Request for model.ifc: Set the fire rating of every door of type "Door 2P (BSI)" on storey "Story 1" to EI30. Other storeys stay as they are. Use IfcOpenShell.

First a look at what the model holds.

```python
import ifcopenshell
import ifcopenshell.util.element

model = ifcopenshell.open("model.ifc")
print(model.schema)
storey = next(s for s in model.by_type("IfcBuildingStorey") if s.Name == "Story 1")
doors = [e for e in ifcopenshell.util.element.get_decomposition(storey) if e.is_a("IfcDoor")]
seen = {}
for e in doors:
    element_type = ifcopenshell.util.element.get_type(e)
    key = (element_type.Name if element_type != e and element_type else None, ifcopenshell.util.element.get_pset(e, "Pset_DoorCommon", "FireRating"))
    seen[key] = seen.get(key, 0) + 1
for (name, value), count in sorted(seen.items(), key=str):
    print(count, "x", name, "|", value)
```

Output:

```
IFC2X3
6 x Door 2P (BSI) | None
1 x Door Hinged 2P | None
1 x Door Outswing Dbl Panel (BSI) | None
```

```python
import ifcopenshell
import ifcopenshell.api.pset
import ifcopenshell.util.element

model = ifcopenshell.open("model.ifc")

storey = next(s for s in model.by_type("IfcBuildingStorey") if s.Name == "Story 1")
doors = [e for e in ifcopenshell.util.element.get_decomposition(storey) if e.is_a("IfcDoor")]

count = 0
for e in doors:
    element_type = ifcopenshell.util.element.get_type(e)
    if element_type in (None, e) or element_type.Name != "Door 2P (BSI)":
        continue
    # add_pset returns the element's existing set when there is one.
    pset = ifcopenshell.api.pset.add_pset(model, product=e, name="Pset_DoorCommon")
    ifcopenshell.api.pset.edit_pset(model, pset=pset, properties={"FireRating": "EI30"})
    count += 1

print(count, "doors updated")

model.write("model_updated.ifc")
```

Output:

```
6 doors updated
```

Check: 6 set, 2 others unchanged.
